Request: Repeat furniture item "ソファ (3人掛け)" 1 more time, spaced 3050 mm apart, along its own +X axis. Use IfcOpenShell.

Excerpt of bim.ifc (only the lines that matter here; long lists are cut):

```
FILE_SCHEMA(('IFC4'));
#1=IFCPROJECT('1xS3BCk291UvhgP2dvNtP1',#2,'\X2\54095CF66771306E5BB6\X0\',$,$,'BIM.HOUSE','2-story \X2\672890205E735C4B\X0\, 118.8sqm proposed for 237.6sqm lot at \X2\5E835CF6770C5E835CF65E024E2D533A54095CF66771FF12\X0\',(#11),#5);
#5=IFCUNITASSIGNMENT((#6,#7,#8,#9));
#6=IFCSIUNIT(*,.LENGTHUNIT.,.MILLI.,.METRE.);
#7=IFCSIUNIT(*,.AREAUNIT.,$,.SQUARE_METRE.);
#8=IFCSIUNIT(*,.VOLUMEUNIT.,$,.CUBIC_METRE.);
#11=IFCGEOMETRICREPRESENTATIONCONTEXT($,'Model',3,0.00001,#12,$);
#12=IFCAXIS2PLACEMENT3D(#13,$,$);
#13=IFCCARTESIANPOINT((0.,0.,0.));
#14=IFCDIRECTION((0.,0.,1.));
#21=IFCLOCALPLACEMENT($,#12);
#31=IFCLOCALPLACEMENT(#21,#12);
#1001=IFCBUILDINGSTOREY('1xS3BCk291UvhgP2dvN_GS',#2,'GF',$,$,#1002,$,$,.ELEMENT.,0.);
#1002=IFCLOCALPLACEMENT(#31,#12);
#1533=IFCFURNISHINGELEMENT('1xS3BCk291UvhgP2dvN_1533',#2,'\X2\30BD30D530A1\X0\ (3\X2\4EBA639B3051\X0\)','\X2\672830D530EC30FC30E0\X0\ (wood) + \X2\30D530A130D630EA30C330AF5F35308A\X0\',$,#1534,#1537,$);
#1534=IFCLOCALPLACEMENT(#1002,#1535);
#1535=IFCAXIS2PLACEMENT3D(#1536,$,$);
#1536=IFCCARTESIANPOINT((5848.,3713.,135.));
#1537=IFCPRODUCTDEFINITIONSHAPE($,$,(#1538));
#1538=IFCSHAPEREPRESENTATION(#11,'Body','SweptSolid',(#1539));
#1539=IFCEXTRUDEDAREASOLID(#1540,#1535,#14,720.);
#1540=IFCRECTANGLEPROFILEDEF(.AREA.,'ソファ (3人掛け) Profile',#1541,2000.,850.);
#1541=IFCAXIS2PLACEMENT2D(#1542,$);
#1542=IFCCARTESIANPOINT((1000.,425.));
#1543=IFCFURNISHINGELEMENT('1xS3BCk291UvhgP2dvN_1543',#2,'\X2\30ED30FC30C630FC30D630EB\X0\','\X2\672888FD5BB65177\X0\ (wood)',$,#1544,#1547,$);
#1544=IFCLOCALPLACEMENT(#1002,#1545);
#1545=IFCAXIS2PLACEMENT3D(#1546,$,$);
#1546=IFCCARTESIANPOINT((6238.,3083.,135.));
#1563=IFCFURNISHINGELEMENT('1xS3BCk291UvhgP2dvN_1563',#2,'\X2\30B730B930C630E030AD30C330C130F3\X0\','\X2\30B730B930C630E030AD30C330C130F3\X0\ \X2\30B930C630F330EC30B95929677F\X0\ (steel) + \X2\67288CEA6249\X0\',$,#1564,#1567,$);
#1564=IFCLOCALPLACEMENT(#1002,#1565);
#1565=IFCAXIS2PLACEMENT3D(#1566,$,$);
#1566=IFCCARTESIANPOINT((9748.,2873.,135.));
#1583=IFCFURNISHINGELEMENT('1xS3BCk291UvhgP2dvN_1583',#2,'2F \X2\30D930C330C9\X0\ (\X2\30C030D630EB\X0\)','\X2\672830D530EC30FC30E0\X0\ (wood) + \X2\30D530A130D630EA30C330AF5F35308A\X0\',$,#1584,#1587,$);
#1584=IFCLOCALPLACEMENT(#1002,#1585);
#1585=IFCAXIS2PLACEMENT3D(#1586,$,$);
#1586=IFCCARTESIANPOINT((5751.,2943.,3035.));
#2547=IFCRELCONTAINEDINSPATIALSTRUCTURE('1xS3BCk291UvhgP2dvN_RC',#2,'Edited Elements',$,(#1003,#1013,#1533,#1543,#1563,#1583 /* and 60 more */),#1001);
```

```python
import ifcopenshell
import ifcopenshell.api.geometry
import ifcopenshell.api.root
import ifcopenshell.util.element
import ifcopenshell.util.placement

model = ifcopenshell.open("bim.ifc")


def reuse_history(source, copy):
    """copy_class also copies each property set's owner history, people and application; keep the originals."""
    for rel in copy.IsDefinedBy:
        if rel.is_a("IfcRelDefinesByProperties") and (history := rel.RelatingPropertyDefinition.OwnerHistory):
            rel.RelatingPropertyDefinition.OwnerHistory = source.OwnerHistory
            ifcopenshell.util.element.remove_deep2(model, history)


source = model.by_guid("1xS3BCk291UvhgP2dvN_1533")
base = ifcopenshell.util.placement.get_local_placement(source.ObjectPlacement)
step = base[:3, 0] * 3050.0

for i in range(1, 2):
    copy = ifcopenshell.api.root.copy_class(model, product=source)
    copy.Representation = ifcopenshell.util.element.copy_deep(
        model, source.Representation, exclude=["IfcGeometricRepresentationContext", "IfcRepresentationMap"]
    )
    reuse_history(source, copy)
    matrix = base.copy()
    matrix[:3, 3] += i * step
    print("added at", matrix[:3, 3].round(3) + 0.0)
    ifcopenshell.api.geometry.edit_object_placement(model, product=copy, matrix=matrix, is_si=False)

model.write("bim-out.ifc")
```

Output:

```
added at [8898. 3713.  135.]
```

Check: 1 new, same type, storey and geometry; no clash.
